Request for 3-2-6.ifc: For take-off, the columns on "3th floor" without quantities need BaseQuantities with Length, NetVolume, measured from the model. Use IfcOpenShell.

First a look at what the model holds.

```python
import ifcopenshell
import ifcopenshell.util.element
import ifcopenshell.util.unit

model = ifcopenshell.open("3-2-6.ifc")
print(model.schema)
for unit_type in ("LENGTHUNIT", "AREAUNIT", "VOLUMEUNIT"):
    print(unit_type, ifcopenshell.util.unit.calculate_unit_scale(model, unit_type))
storey = next(s for s in model.by_type("IfcBuildingStorey") if s.Name == "3th floor")
columns = [e for e in ifcopenshell.util.element.get_decomposition(storey) if e.is_a("IfcColumn")]
for e in sorted(columns, key=lambda e: e.id()):
    print(e.id(), e.is_a(), e.Name, list(ifcopenshell.util.element.get_psets(e, qtos_only=True)), sep=" | ")
```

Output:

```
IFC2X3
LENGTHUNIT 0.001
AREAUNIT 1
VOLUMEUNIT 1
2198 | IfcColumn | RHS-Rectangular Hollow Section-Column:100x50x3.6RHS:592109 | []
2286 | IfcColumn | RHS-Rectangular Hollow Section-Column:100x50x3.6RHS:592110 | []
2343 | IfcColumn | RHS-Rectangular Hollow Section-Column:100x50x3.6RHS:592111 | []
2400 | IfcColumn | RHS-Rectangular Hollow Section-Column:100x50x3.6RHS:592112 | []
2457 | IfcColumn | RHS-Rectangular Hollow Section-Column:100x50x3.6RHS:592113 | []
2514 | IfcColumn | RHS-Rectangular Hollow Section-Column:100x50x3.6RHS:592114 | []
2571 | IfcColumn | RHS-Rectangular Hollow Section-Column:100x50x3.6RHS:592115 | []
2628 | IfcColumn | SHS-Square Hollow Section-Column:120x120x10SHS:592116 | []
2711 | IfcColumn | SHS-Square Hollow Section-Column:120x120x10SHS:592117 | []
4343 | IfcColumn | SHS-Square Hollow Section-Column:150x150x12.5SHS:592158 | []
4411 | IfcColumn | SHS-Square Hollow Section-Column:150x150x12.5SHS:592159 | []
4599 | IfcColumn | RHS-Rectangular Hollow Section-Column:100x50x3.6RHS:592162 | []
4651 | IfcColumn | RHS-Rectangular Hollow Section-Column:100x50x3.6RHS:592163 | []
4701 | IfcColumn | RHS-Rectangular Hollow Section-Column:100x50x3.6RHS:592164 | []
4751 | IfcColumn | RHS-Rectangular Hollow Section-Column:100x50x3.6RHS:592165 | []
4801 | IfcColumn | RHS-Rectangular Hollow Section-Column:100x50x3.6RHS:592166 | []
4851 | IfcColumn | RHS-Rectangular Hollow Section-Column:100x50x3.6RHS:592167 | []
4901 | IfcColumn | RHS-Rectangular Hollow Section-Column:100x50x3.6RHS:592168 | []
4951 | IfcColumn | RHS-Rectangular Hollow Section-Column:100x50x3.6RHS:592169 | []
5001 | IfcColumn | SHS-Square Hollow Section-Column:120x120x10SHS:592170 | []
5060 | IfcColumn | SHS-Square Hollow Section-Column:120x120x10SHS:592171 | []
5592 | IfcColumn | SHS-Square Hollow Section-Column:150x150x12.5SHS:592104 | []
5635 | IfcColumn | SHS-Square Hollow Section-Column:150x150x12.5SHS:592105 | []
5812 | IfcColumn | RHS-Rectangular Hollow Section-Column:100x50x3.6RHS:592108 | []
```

```python
import ifcopenshell
import ifcopenshell.api.pset
import ifcopenshell.geom
import ifcopenshell.util.element
import ifcopenshell.util.shape
import ifcopenshell.util.unit

model = ifcopenshell.open("3-2-6.ifc")
unit_scale = ifcopenshell.util.unit.calculate_unit_scale(model)
volume_scale = ifcopenshell.util.unit.calculate_unit_scale(model, "VOLUMEUNIT")
settings = ifcopenshell.geom.settings()

storey = next(s for s in model.by_type("IfcBuildingStorey") if s.Name == "3th floor")
columns = [e for e in ifcopenshell.util.element.get_decomposition(storey) if e.is_a("IfcColumn")]

for e in sorted(columns, key=lambda e: e.id()):
    if ifcopenshell.util.element.get_psets(e, qtos_only=True, should_inherit=False):
        continue
    # Geometry comes back in metres, in the element's own axes.
    shape = ifcopenshell.geom.create_shape(settings, e)
    values = {
        "Length": ifcopenshell.util.shape.get_z(shape.geometry) / unit_scale,
        "NetVolume": ifcopenshell.util.shape.get_volume(shape.geometry) / volume_scale,
    }
    qto = ifcopenshell.api.pset.add_qto(model, product=e, name="BaseQuantities")
    ifcopenshell.api.pset.edit_qto(model, qto=qto, properties=values)
    print(e.id(), {k: round(v, 3) for k, v in values.items()})

model.write("3-2-6_updated.ifc")
```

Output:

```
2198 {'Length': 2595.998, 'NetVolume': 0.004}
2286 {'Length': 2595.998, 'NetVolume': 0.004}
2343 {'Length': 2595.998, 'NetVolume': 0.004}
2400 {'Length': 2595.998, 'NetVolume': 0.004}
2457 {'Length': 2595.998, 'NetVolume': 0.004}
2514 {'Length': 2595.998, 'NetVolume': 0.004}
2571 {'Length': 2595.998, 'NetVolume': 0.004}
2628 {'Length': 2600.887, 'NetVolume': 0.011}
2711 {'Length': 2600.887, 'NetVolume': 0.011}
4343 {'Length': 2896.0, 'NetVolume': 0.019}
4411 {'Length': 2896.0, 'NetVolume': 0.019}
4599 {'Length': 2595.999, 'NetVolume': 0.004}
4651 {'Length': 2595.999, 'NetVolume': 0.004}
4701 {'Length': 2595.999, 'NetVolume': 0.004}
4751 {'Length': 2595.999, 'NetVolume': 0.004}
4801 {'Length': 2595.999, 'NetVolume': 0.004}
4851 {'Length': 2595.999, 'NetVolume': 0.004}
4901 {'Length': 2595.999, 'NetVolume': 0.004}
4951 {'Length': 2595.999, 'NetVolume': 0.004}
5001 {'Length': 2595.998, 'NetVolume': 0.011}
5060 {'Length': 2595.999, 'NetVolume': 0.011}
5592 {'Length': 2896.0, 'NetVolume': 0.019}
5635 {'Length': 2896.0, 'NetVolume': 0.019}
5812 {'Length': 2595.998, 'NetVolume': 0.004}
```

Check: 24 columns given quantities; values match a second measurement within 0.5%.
